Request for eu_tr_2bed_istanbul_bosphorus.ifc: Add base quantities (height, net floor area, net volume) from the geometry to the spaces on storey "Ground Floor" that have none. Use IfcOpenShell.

First a look at what the model holds.

```python
import ifcopenshell
import ifcopenshell.util.element
import ifcopenshell.util.unit

model = ifcopenshell.open("eu_tr_2bed_istanbul_bosphorus.ifc")
print(model.schema)
for unit_type in ("LENGTHUNIT", "AREAUNIT", "VOLUMEUNIT"):
    print(unit_type, ifcopenshell.util.unit.calculate_unit_scale(model, unit_type))
storey = next(s for s in model.by_type("IfcBuildingStorey") if s.Name == "Ground Floor")
spaces = [e for e in ifcopenshell.util.element.get_decomposition(storey) if e.is_a("IfcSpace")]
for e in sorted(spaces, key=lambda e: e.id()):
    print(e.id(), e.is_a(), e.Name, list(ifcopenshell.util.element.get_psets(e, qtos_only=True)), sep=" | ")
```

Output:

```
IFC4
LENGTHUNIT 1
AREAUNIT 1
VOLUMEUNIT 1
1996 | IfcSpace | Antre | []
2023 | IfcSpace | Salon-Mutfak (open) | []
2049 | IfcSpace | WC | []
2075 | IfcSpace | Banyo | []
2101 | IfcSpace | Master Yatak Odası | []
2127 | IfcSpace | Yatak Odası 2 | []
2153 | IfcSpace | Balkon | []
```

```python
import ifcopenshell
import ifcopenshell.api.pset
import ifcopenshell.geom
import ifcopenshell.util.element
import ifcopenshell.util.shape
import ifcopenshell.util.unit

model = ifcopenshell.open("eu_tr_2bed_istanbul_bosphorus.ifc")
unit_scale = ifcopenshell.util.unit.calculate_unit_scale(model)
area_scale = ifcopenshell.util.unit.calculate_unit_scale(model, "AREAUNIT")
volume_scale = ifcopenshell.util.unit.calculate_unit_scale(model, "VOLUMEUNIT")
settings = ifcopenshell.geom.settings()

storey = next(s for s in model.by_type("IfcBuildingStorey") if s.Name == "Ground Floor")
spaces = [e for e in ifcopenshell.util.element.get_decomposition(storey) if e.is_a("IfcSpace")]

for e in sorted(spaces, key=lambda e: e.id()):
    if ifcopenshell.util.element.get_psets(e, qtos_only=True, should_inherit=False):
        continue
    # Geometry comes back in metres, in the element's own axes.
    shape = ifcopenshell.geom.create_shape(settings, e)
    values = {
        "Height": ifcopenshell.util.shape.get_z(shape.geometry) / unit_scale,
        "NetFloorArea": ifcopenshell.util.shape.get_footprint_area(shape.geometry) / area_scale,
        "NetVolume": ifcopenshell.util.shape.get_volume(shape.geometry) / volume_scale,
    }
    qto = ifcopenshell.api.pset.add_qto(model, product=e, name="Qto_SpaceBaseQuantities")
    ifcopenshell.api.pset.edit_qto(model, qto=qto, properties=values)
    print(e.id(), {k: round(v, 3) for k, v in values.items()})

model.write("eu_tr_2bed_istanbul_bosphorus_updated.ifc")
```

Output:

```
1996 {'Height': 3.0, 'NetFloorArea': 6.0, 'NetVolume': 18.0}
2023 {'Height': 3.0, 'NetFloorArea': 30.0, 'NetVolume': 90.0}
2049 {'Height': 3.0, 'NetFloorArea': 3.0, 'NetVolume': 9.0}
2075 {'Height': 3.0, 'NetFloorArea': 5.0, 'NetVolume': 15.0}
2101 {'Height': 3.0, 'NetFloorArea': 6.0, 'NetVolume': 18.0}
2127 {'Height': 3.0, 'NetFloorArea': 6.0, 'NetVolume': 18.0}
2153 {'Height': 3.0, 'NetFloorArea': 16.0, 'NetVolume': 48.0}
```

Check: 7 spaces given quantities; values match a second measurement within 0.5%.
